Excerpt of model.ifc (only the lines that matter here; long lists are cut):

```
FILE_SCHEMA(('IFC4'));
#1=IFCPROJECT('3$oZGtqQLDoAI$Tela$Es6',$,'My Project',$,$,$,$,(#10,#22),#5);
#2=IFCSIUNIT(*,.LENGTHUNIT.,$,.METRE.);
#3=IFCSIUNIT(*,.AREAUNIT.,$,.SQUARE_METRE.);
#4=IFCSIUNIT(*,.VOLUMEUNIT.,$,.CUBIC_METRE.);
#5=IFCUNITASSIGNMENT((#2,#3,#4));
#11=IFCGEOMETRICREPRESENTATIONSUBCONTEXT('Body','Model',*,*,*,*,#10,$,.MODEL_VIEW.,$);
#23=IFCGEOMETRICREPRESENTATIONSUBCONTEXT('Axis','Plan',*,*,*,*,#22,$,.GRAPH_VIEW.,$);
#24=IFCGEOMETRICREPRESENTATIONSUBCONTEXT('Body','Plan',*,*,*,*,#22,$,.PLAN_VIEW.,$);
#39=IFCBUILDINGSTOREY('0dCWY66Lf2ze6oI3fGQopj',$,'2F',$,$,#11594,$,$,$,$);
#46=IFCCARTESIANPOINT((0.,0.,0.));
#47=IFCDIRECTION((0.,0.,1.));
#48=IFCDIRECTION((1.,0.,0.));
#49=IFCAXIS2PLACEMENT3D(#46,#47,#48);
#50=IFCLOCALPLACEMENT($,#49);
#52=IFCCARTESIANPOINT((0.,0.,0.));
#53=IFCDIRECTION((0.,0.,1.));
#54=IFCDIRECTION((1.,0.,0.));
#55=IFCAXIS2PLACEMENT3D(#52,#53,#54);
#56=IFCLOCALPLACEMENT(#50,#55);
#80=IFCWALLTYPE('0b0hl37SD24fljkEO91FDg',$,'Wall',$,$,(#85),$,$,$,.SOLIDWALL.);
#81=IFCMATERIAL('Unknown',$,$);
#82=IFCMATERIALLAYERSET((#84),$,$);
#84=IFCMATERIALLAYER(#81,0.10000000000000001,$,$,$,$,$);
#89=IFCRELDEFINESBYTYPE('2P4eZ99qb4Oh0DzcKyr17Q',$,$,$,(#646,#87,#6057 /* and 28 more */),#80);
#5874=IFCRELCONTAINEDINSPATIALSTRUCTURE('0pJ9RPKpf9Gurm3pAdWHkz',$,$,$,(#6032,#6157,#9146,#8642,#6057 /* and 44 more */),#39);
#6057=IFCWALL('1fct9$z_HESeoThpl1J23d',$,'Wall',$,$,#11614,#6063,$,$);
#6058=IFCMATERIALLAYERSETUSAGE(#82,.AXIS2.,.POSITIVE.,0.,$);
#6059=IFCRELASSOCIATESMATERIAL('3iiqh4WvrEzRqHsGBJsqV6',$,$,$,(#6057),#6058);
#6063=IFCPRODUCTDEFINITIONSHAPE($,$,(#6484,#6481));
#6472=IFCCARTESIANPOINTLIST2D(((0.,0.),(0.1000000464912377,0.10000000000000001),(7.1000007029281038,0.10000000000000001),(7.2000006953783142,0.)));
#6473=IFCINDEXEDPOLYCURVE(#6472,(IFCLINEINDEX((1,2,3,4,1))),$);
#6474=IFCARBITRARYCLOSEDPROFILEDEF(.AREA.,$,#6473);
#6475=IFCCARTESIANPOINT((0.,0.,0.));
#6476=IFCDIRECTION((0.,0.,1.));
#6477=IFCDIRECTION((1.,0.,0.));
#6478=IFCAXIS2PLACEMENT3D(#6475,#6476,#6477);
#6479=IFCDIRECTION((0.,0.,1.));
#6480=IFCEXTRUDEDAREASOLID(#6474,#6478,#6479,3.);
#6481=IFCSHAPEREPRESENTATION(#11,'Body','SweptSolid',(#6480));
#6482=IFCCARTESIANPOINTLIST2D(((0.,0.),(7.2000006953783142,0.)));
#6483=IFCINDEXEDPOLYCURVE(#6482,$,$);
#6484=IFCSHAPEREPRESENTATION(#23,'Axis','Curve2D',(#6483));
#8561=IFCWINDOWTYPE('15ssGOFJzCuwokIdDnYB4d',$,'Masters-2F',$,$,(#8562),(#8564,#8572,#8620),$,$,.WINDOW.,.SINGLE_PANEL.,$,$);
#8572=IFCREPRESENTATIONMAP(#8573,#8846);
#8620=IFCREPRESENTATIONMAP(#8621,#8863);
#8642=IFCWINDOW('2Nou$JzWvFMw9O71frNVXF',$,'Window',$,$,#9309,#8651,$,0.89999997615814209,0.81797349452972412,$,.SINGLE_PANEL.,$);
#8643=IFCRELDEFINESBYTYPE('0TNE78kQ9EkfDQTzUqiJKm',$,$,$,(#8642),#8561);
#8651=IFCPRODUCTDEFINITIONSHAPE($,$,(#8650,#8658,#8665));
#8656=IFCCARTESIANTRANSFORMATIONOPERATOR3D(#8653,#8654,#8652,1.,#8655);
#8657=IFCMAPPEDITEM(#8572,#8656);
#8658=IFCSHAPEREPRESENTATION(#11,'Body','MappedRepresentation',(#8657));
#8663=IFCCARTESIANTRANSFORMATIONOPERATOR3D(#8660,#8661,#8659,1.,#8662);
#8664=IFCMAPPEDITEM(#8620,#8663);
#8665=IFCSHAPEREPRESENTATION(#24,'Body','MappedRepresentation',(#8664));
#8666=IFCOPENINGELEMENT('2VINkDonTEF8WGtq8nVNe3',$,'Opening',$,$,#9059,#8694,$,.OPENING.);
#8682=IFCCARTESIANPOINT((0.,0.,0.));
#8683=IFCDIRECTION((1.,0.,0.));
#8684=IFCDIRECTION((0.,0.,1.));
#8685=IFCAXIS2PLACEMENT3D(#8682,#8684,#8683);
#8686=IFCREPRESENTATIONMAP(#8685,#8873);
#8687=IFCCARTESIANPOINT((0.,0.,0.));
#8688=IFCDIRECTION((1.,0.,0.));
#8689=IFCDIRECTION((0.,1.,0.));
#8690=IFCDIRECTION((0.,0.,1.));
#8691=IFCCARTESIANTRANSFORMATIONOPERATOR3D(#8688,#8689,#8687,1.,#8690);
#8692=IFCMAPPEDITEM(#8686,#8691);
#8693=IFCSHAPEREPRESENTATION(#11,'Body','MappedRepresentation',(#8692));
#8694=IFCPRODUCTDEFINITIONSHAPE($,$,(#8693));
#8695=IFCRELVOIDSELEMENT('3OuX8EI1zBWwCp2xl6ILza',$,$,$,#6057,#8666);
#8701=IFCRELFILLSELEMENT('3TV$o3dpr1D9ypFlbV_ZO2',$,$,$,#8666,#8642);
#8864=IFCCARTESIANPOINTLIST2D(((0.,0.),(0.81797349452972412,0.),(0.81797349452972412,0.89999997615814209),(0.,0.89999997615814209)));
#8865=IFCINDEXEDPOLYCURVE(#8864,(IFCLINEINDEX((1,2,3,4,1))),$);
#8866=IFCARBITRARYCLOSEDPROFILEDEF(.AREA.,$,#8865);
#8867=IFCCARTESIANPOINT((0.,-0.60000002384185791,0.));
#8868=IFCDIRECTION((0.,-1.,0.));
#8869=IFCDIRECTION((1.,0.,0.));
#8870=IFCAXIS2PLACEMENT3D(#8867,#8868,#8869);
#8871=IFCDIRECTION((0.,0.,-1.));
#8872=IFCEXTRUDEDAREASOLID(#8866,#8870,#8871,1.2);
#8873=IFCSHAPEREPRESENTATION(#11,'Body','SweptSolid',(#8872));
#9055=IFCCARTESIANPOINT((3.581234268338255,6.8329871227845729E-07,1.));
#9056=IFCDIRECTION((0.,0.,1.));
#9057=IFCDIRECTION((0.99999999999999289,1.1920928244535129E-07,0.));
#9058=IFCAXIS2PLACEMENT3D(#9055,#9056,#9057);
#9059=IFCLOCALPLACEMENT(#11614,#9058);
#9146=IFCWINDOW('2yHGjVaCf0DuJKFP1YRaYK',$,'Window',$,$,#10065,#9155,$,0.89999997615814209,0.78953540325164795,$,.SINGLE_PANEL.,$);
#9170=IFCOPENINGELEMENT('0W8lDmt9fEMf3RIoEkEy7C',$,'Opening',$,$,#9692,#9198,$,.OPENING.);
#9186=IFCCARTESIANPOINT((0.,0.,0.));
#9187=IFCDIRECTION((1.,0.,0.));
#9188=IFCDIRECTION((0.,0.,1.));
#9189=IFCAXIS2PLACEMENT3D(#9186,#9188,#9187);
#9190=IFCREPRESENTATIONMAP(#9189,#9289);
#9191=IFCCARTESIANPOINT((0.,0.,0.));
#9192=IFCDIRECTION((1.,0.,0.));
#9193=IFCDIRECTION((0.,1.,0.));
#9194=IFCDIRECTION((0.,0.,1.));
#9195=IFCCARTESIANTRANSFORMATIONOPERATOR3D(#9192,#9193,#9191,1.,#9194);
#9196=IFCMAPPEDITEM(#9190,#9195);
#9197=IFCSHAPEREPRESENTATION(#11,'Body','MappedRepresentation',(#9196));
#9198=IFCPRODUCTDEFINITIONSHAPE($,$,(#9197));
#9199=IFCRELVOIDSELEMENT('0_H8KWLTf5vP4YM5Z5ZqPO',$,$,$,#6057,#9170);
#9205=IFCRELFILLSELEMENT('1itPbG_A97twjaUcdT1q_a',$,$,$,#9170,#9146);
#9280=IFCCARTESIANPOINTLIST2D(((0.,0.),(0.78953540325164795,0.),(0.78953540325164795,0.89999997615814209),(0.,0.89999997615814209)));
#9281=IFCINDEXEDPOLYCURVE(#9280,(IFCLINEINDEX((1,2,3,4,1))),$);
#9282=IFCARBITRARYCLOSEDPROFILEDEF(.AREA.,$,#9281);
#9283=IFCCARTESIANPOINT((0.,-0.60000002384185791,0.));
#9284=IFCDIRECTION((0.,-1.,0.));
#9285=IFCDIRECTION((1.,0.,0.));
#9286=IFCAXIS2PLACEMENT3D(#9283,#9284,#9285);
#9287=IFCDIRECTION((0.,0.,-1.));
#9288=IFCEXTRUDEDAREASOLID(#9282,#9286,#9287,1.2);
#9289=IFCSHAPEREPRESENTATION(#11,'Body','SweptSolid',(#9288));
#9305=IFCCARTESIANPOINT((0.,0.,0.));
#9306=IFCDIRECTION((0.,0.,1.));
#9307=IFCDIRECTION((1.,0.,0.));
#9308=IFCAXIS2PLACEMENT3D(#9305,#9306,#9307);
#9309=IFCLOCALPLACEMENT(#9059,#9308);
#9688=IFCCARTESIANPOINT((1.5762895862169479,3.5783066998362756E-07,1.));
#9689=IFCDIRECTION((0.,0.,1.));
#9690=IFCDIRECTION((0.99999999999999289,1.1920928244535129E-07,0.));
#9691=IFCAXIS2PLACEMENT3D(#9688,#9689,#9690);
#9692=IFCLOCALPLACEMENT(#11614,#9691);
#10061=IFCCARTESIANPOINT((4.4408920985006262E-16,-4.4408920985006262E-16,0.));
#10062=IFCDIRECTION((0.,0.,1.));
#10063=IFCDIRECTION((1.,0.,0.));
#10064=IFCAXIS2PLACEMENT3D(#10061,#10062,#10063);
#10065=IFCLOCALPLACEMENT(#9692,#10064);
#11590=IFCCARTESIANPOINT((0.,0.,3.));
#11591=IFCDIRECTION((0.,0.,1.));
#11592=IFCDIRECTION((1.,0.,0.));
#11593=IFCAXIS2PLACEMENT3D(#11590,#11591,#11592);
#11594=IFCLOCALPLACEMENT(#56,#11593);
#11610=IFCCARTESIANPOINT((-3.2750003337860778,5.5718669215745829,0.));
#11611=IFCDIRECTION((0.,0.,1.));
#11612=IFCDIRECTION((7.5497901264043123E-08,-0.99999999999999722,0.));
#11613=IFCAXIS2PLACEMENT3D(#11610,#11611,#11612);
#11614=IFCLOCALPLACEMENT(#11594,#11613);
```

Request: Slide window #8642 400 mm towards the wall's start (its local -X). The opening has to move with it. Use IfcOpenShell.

```python
import ifcopenshell
import ifcopenshell.api.geometry
import ifcopenshell.util.placement
import ifcopenshell.util.unit

model = ifcopenshell.open("model.ifc")
unit_scale = ifcopenshell.util.unit.calculate_unit_scale(model)

window = model.by_guid("2Nou$JzWvFMw9O71frNVXF")
opening = window.FillsVoids[0].RelatingOpeningElement
wall = opening.VoidsElements[0].RelatingBuildingElement

wall_matrix = ifcopenshell.util.placement.get_local_placement(wall.ObjectPlacement)
shift = wall_matrix[:3, 0] * -0.4 / unit_scale
before = ifcopenshell.util.placement.get_local_placement(window.ObjectPlacement)[:3, 3].copy()

# The window is placed relative to its opening, so it follows when the opening moves.
matrix = ifcopenshell.util.placement.get_local_placement(opening.ObjectPlacement)
matrix[:3, 3] += shift
ifcopenshell.api.geometry.edit_object_placement(
    model, product=opening, matrix=matrix, is_si=False, should_transform_children=True
)

after = ifcopenshell.util.placement.get_local_placement(window.ObjectPlacement)[:3, 3]
print("window moved by", (after - before).round(3) + 0.0)

model.write("model_updated.ifc")
```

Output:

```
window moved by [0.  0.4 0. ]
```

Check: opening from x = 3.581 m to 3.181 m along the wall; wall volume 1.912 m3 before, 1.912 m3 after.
